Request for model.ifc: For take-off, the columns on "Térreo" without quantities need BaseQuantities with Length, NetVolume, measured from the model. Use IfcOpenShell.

First a look at what the model holds.

```python
import ifcopenshell
import ifcopenshell.util.element
import ifcopenshell.util.unit

model = ifcopenshell.open("model.ifc")
print(model.schema)
for unit_type in ("LENGTHUNIT", "AREAUNIT", "VOLUMEUNIT"):
    print(unit_type, ifcopenshell.util.unit.calculate_unit_scale(model, unit_type))
storey = next(s for s in model.by_type("IfcBuildingStorey") if s.Name == "Térreo")
columns = [e for e in ifcopenshell.util.element.get_decomposition(storey) if e.is_a("IfcColumn")]
for e in sorted(columns, key=lambda e: e.id()):
    print(e.id(), e.is_a(), e.Name, list(ifcopenshell.util.element.get_psets(e, qtos_only=True)), sep=" | ")
```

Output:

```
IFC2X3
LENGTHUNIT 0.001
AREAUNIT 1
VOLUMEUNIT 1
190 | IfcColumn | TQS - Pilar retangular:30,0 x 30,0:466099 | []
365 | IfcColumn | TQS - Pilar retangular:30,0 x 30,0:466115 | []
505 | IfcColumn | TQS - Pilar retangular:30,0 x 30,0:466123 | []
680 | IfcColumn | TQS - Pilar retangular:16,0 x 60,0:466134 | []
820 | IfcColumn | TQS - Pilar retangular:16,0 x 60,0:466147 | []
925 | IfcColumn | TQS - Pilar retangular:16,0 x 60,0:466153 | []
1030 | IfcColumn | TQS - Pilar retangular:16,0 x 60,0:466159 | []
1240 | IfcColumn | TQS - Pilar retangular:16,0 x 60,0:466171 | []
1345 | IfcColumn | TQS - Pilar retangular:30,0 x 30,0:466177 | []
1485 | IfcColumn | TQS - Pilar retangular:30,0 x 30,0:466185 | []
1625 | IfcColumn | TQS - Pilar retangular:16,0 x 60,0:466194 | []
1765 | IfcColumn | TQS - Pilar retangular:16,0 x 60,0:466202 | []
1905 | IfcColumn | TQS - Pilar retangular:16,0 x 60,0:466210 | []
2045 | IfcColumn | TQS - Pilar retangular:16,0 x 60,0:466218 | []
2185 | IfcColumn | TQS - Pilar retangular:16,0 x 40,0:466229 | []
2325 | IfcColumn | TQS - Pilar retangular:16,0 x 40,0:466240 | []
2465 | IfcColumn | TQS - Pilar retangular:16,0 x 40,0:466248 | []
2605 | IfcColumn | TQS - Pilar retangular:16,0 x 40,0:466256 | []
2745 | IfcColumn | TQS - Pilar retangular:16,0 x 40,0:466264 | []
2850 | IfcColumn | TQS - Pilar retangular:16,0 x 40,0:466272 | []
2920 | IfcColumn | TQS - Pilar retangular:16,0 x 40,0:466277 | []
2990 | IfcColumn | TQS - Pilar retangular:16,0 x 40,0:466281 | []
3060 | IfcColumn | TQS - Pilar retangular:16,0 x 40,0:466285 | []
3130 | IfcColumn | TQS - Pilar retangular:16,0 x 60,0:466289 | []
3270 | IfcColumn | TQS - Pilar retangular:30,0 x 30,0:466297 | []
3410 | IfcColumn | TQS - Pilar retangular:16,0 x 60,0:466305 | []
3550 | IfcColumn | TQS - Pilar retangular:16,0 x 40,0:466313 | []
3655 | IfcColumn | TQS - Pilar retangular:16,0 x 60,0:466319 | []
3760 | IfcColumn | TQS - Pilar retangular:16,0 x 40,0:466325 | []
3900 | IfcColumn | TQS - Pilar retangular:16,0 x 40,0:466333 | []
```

```python
import ifcopenshell
import ifcopenshell.api.pset
import ifcopenshell.geom
import ifcopenshell.util.element
import ifcopenshell.util.shape
import ifcopenshell.util.unit

model = ifcopenshell.open("model.ifc")
unit_scale = ifcopenshell.util.unit.calculate_unit_scale(model)
volume_scale = ifcopenshell.util.unit.calculate_unit_scale(model, "VOLUMEUNIT")
settings = ifcopenshell.geom.settings()

storey = next(s for s in model.by_type("IfcBuildingStorey") if s.Name == "Térreo")
columns = [e for e in ifcopenshell.util.element.get_decomposition(storey) if e.is_a("IfcColumn")]

for e in sorted(columns, key=lambda e: e.id()):
    if ifcopenshell.util.element.get_psets(e, qtos_only=True, should_inherit=False):
        continue
    # Geometry comes back in metres, in the element's own axes.
    shape = ifcopenshell.geom.create_shape(settings, e)
    values = {
        "Length": ifcopenshell.util.shape.get_z(shape.geometry) / unit_scale,
        "NetVolume": ifcopenshell.util.shape.get_volume(shape.geometry) / volume_scale,
    }
    qto = ifcopenshell.api.pset.add_qto(model, product=e, name="BaseQuantities")
    ifcopenshell.api.pset.edit_qto(model, qto=qto, properties=values)
    print(e.id(), {k: round(v, 3) for k, v in values.items()})

model.write("model-out.ifc")
```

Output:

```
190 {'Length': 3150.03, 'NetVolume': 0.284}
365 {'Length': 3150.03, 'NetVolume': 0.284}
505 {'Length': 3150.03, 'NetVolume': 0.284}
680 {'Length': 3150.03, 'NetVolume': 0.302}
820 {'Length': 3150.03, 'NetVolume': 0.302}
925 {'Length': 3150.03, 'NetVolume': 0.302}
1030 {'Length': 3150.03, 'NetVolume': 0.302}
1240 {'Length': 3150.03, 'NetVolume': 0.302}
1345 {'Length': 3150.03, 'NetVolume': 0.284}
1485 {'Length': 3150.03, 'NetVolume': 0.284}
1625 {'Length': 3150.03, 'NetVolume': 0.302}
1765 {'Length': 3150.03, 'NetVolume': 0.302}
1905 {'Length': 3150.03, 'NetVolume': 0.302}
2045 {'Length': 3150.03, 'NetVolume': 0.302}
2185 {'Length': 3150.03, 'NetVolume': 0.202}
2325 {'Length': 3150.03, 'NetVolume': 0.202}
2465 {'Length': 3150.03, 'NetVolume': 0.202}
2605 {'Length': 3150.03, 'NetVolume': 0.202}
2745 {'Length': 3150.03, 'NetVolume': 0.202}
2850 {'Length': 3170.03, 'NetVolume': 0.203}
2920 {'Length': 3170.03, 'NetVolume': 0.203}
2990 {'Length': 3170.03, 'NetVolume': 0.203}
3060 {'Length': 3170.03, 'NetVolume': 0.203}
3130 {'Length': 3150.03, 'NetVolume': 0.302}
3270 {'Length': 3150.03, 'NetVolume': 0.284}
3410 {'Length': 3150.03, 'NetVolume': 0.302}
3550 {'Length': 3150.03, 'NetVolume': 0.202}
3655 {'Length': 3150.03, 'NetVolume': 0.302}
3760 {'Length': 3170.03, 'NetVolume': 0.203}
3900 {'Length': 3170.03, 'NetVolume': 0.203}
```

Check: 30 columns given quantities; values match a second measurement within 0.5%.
